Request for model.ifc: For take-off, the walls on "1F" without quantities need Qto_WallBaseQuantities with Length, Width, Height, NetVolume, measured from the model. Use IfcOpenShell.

First a look at what the model holds.

```python
import ifcopenshell
import ifcopenshell.util.element
import ifcopenshell.util.unit

model = ifcopenshell.open("model.ifc")
print(model.schema)
for unit_type in ("LENGTHUNIT", "AREAUNIT", "VOLUMEUNIT"):
    print(unit_type, ifcopenshell.util.unit.calculate_unit_scale(model, unit_type))
storey = next(s for s in model.by_type("IfcBuildingStorey") if s.Name == "1F")
walls = [e for e in ifcopenshell.util.element.get_decomposition(storey) if e.is_a("IfcWall")]
for e in sorted(walls, key=lambda e: e.id()):
    print(e.id(), e.is_a(), e.Name, list(ifcopenshell.util.element.get_psets(e, qtos_only=True)), sep=" | ")
```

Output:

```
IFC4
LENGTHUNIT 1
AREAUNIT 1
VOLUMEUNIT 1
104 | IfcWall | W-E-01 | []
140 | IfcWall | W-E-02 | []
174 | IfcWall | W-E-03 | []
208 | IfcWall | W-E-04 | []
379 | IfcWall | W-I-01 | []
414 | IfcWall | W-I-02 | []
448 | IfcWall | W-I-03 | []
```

```python
import ifcopenshell
import ifcopenshell.api.pset
import ifcopenshell.geom
import ifcopenshell.util.element
import ifcopenshell.util.shape
import ifcopenshell.util.unit

model = ifcopenshell.open("model.ifc")
unit_scale = ifcopenshell.util.unit.calculate_unit_scale(model)
volume_scale = ifcopenshell.util.unit.calculate_unit_scale(model, "VOLUMEUNIT")
settings = ifcopenshell.geom.settings()

storey = next(s for s in model.by_type("IfcBuildingStorey") if s.Name == "1F")
walls = [e for e in ifcopenshell.util.element.get_decomposition(storey) if e.is_a("IfcWall")]

for e in sorted(walls, key=lambda e: e.id()):
    if ifcopenshell.util.element.get_psets(e, qtos_only=True, should_inherit=False):
        continue
    # Geometry comes back in metres, in the element's own axes.
    shape = ifcopenshell.geom.create_shape(settings, e)
    values = {
        "Length": ifcopenshell.util.shape.get_x(shape.geometry) / unit_scale,
        "Width": ifcopenshell.util.shape.get_y(shape.geometry) / unit_scale,
        "Height": ifcopenshell.util.shape.get_z(shape.geometry) / unit_scale,
        "NetVolume": ifcopenshell.util.shape.get_volume(shape.geometry) / volume_scale,
    }
    qto = ifcopenshell.api.pset.add_qto(model, product=e, name="Qto_WallBaseQuantities")
    ifcopenshell.api.pset.edit_qto(model, qto=qto, properties=values)
    print(e.id(), {k: round(v, 3) for k, v in values.items()})

model.write("model_rev.ifc")
```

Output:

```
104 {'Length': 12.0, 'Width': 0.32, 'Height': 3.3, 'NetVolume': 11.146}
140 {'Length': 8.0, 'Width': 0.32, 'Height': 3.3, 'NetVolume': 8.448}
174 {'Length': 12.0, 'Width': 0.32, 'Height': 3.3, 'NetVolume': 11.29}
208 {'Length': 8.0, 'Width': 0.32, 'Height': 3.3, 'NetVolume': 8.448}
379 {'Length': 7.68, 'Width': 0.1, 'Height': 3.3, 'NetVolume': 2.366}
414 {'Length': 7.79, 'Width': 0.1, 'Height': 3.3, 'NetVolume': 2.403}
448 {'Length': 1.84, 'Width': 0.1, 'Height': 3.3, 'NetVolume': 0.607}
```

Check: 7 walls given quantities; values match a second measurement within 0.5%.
